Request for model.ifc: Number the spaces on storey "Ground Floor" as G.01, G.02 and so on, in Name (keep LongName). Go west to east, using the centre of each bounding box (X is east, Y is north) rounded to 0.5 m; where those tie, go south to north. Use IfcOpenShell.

First a look at what the model holds.

```python
import ifcopenshell
import ifcopenshell.util.element
import ifcopenshell.util.placement

model = ifcopenshell.open("model.ifc")
print(model.schema)
storey = next(s for s in model.by_type("IfcBuildingStorey") if s.Name == "Ground Floor")
spaces = [e for e in ifcopenshell.util.element.get_decomposition(storey) if e.is_a("IfcSpace")]
for e in sorted(spaces, key=lambda e: e.id()):
    origin = ifcopenshell.util.placement.get_local_placement(e.ObjectPlacement)[:3, 3]
    print(e.id(), e.Name, e.LongName, origin.round(2) + 0.0, sep=" | ")
```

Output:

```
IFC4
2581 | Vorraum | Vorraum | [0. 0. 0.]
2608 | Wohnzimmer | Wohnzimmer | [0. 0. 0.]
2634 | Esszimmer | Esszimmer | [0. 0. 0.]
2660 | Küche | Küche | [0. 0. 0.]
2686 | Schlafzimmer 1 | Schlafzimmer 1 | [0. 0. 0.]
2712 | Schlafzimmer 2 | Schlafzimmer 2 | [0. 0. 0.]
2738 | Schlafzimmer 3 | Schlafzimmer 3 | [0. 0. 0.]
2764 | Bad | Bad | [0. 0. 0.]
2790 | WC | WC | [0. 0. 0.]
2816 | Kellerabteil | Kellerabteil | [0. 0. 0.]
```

```python
import ifcopenshell
import ifcopenshell.geom
import ifcopenshell.util.element
import ifcopenshell.util.shape

model = ifcopenshell.open("model.ifc")
settings = ifcopenshell.geom.settings()
settings.set("use-world-coords", True)


def centre(element):
    shape = ifcopenshell.geom.create_shape(settings, element)
    return ifcopenshell.util.shape.get_bbox_centroid(shape.geometry)


storey = next(s for s in model.by_type("IfcBuildingStorey") if s.Name == "Ground Floor")
spaces = [e for e in ifcopenshell.util.element.get_decomposition(storey) if e.is_a("IfcSpace")]

# Insertion points can sit at a corner or the storey origin, so sort by the geometry (in metres).
centres = {e: centre(e) for e in spaces}
spaces.sort(key=lambda e: (round(centres[e][0] / 0.5), centres[e][1]))

for i, e in enumerate(spaces, start=1):
    number = f"G.{i:02d}"
    e.Name = number
    print(e.id(), number)

model.write("model_rev.ifc")
```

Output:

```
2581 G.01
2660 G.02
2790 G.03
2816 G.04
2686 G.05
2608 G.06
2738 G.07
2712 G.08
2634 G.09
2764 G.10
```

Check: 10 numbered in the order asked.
